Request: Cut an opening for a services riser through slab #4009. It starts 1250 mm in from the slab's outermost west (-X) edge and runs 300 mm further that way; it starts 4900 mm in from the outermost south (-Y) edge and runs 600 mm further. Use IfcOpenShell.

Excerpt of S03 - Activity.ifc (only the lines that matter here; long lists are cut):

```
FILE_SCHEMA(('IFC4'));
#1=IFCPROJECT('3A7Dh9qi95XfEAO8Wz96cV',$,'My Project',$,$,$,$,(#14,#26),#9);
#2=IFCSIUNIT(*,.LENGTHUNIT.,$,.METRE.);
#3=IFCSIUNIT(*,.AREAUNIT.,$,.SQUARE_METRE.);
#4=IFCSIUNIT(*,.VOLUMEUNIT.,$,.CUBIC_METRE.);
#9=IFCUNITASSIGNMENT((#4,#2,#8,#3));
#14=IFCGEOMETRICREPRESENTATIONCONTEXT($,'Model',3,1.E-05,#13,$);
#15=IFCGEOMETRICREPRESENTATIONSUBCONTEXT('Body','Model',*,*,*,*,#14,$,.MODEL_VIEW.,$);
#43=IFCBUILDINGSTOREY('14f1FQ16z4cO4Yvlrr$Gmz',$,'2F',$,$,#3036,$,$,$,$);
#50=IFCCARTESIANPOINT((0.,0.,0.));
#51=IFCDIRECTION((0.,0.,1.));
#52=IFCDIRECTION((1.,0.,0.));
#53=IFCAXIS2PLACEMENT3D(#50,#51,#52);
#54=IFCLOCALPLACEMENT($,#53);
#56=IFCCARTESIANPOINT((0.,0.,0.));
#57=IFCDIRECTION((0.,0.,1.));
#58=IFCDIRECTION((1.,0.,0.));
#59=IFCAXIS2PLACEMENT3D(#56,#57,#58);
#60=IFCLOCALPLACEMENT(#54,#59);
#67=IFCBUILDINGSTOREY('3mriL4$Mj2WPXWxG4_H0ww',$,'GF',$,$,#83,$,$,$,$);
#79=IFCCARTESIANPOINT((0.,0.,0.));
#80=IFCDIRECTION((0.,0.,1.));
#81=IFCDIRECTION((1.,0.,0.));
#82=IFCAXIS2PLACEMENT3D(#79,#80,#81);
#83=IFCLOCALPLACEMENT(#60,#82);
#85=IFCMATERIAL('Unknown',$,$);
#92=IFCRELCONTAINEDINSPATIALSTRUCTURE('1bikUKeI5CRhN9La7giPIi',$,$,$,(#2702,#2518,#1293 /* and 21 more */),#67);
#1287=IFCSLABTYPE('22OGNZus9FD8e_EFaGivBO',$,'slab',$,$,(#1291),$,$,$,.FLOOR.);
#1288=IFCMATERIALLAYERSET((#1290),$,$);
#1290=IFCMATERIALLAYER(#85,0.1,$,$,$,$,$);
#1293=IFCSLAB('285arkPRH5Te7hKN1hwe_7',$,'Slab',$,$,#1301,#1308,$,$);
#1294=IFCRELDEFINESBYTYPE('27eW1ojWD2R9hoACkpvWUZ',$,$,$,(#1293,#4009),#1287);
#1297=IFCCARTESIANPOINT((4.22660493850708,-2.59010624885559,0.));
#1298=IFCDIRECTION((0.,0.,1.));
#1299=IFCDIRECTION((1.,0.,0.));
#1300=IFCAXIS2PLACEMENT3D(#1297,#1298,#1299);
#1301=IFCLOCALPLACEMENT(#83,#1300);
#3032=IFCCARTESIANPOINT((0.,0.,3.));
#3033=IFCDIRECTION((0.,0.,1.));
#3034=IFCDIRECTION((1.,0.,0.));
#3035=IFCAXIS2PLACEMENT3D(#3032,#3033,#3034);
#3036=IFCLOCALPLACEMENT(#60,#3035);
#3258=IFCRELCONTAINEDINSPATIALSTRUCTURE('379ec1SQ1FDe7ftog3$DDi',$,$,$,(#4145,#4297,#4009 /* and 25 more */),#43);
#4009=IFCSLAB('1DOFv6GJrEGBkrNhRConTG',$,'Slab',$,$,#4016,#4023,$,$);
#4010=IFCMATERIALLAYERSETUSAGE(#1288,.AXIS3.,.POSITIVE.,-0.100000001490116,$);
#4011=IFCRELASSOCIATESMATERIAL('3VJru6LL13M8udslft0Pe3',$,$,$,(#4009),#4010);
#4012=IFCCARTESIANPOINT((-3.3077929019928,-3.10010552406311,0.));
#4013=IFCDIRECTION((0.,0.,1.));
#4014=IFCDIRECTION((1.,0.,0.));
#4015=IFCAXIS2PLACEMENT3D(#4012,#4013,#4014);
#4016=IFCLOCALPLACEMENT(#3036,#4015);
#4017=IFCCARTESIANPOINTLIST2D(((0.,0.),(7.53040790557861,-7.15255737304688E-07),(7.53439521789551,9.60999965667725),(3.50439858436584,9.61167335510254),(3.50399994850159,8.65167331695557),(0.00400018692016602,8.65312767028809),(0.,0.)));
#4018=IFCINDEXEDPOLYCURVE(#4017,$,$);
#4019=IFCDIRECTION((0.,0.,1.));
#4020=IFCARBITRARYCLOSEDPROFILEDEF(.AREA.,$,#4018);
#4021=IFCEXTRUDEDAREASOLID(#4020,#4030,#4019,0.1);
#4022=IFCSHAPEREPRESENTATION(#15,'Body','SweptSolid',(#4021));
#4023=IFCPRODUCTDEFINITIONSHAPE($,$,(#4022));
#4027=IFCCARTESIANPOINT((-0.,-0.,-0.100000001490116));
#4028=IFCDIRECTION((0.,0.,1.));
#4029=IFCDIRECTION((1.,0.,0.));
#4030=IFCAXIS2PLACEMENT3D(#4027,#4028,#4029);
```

```python
import numpy as np
import ifcopenshell
import ifcopenshell.api.feature
import ifcopenshell.api.geometry
import ifcopenshell.api.root
import ifcopenshell.geom
import ifcopenshell.util.placement
import ifcopenshell.util.representation
import ifcopenshell.util.shape
import ifcopenshell.util.unit

model = ifcopenshell.open("S03 - Activity.ifc")
unit_scale = ifcopenshell.util.unit.calculate_unit_scale(model)
settings = ifcopenshell.geom.settings()


def volume(element):
    """Net volume in cubic metres, openings subtracted."""
    shape = ifcopenshell.geom.create_shape(settings, element)
    return ifcopenshell.util.shape.get_volume(shape.geometry)


slab = model.by_guid("1DOFv6GJrEGBkrNhRConTG")
before = volume(slab)

# Extent in the slab's own axes, in metres. The edges named are its -X and -Y sides.
slab_shape = ifcopenshell.geom.create_shape(settings, slab)
vertices = ifcopenshell.util.shape.get_vertices(slab_shape.geometry)
x_min, y_min, bottom = vertices.min(axis=0)
top = vertices[:, 2].max()

opening = ifcopenshell.api.root.create_entity(model, ifc_class="IfcOpeningElement", name="Services riser opening", predefined_type="OPENING")
context = ifcopenshell.util.representation.get_context(model, "Model", "Body", "MODEL_VIEW")
width, depth = 0.3, 0.6
outline = [(0.0, 0.0), (width, 0.0), (width, depth), (0.0, depth), (0.0, 0.0)]
# Overshoot both faces by 50 mm so the cut is clean.
shape = ifcopenshell.api.geometry.add_slab_representation(
    model, context=context, depth=top - bottom + 0.1, polyline=outline
)
ifcopenshell.api.geometry.assign_representation(model, product=opening, representation=shape)

matrix = ifcopenshell.util.placement.get_local_placement(slab.ObjectPlacement)
matrix[:, 3] = matrix @ np.append(np.array([x_min + 1.25, y_min + 4.9, bottom - 0.05]) / unit_scale, 1.0)
ifcopenshell.api.geometry.edit_object_placement(model, product=opening, matrix=matrix, is_si=False)
ifcopenshell.api.feature.add_feature(model, feature=opening, element=slab)

after = volume(slab)

print(f"slab volume {before:.3f} -> {after:.3f} m3")

model.write("S03 - Activity-out.ifc")
```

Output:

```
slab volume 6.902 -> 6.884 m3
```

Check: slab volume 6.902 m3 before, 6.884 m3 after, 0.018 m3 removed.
